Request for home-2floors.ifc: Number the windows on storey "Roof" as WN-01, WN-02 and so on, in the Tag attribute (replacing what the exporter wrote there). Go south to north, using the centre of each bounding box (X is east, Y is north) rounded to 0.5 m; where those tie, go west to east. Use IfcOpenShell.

First a look at what the model holds.

```python
import ifcopenshell
import ifcopenshell.util.element
import ifcopenshell.util.placement

model = ifcopenshell.open("home-2floors.ifc")
print(model.schema)
storey = next(s for s in model.by_type("IfcBuildingStorey") if s.Name == "Roof")
windows = [e for e in ifcopenshell.util.element.get_decomposition(storey) if e.is_a("IfcWindow")]
for e in sorted(windows, key=lambda e: e.id()):
    origin = ifcopenshell.util.placement.get_local_placement(e.ObjectPlacement)[:3, 3]
    print(e.id(), e.Tag, e.Name, origin.round(2) + 0.0, sep=" | ")
```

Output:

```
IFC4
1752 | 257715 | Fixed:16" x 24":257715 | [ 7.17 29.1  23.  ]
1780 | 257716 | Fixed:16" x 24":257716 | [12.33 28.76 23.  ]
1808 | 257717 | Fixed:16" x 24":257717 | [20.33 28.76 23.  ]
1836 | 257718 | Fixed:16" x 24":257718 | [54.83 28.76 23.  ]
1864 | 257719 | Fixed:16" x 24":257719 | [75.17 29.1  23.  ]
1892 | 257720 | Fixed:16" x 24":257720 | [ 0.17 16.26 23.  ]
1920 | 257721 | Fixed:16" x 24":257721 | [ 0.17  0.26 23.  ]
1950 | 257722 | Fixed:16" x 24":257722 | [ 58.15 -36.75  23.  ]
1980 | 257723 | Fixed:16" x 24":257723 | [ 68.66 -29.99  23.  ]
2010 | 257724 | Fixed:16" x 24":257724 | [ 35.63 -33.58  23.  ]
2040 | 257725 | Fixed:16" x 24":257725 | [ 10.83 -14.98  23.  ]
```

```python
import ifcopenshell
import ifcopenshell.geom
import ifcopenshell.util.element
import ifcopenshell.util.shape

model = ifcopenshell.open("home-2floors.ifc")
settings = ifcopenshell.geom.settings()
settings.set("use-world-coords", True)


def centre(element):
    shape = ifcopenshell.geom.create_shape(settings, element)
    return ifcopenshell.util.shape.get_bbox_centroid(shape.geometry)


storey = next(s for s in model.by_type("IfcBuildingStorey") if s.Name == "Roof")
windows = [e for e in ifcopenshell.util.element.get_decomposition(storey) if e.is_a("IfcWindow")]

# Insertion points can sit at a corner or the storey origin, so sort by the geometry (in metres).
centres = {e: centre(e) for e in windows}
windows.sort(key=lambda e: (round(centres[e][1] / 0.5), centres[e][0]))

for i, e in enumerate(windows, start=1):
    number = f"WN-{i:02d}"
    e.Tag = number
    print(e.id(), number)

model.write("home-2floors_edited.ifc")
```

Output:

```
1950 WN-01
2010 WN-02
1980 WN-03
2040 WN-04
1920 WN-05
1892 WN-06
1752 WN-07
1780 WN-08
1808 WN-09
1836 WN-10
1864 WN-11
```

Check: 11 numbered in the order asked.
